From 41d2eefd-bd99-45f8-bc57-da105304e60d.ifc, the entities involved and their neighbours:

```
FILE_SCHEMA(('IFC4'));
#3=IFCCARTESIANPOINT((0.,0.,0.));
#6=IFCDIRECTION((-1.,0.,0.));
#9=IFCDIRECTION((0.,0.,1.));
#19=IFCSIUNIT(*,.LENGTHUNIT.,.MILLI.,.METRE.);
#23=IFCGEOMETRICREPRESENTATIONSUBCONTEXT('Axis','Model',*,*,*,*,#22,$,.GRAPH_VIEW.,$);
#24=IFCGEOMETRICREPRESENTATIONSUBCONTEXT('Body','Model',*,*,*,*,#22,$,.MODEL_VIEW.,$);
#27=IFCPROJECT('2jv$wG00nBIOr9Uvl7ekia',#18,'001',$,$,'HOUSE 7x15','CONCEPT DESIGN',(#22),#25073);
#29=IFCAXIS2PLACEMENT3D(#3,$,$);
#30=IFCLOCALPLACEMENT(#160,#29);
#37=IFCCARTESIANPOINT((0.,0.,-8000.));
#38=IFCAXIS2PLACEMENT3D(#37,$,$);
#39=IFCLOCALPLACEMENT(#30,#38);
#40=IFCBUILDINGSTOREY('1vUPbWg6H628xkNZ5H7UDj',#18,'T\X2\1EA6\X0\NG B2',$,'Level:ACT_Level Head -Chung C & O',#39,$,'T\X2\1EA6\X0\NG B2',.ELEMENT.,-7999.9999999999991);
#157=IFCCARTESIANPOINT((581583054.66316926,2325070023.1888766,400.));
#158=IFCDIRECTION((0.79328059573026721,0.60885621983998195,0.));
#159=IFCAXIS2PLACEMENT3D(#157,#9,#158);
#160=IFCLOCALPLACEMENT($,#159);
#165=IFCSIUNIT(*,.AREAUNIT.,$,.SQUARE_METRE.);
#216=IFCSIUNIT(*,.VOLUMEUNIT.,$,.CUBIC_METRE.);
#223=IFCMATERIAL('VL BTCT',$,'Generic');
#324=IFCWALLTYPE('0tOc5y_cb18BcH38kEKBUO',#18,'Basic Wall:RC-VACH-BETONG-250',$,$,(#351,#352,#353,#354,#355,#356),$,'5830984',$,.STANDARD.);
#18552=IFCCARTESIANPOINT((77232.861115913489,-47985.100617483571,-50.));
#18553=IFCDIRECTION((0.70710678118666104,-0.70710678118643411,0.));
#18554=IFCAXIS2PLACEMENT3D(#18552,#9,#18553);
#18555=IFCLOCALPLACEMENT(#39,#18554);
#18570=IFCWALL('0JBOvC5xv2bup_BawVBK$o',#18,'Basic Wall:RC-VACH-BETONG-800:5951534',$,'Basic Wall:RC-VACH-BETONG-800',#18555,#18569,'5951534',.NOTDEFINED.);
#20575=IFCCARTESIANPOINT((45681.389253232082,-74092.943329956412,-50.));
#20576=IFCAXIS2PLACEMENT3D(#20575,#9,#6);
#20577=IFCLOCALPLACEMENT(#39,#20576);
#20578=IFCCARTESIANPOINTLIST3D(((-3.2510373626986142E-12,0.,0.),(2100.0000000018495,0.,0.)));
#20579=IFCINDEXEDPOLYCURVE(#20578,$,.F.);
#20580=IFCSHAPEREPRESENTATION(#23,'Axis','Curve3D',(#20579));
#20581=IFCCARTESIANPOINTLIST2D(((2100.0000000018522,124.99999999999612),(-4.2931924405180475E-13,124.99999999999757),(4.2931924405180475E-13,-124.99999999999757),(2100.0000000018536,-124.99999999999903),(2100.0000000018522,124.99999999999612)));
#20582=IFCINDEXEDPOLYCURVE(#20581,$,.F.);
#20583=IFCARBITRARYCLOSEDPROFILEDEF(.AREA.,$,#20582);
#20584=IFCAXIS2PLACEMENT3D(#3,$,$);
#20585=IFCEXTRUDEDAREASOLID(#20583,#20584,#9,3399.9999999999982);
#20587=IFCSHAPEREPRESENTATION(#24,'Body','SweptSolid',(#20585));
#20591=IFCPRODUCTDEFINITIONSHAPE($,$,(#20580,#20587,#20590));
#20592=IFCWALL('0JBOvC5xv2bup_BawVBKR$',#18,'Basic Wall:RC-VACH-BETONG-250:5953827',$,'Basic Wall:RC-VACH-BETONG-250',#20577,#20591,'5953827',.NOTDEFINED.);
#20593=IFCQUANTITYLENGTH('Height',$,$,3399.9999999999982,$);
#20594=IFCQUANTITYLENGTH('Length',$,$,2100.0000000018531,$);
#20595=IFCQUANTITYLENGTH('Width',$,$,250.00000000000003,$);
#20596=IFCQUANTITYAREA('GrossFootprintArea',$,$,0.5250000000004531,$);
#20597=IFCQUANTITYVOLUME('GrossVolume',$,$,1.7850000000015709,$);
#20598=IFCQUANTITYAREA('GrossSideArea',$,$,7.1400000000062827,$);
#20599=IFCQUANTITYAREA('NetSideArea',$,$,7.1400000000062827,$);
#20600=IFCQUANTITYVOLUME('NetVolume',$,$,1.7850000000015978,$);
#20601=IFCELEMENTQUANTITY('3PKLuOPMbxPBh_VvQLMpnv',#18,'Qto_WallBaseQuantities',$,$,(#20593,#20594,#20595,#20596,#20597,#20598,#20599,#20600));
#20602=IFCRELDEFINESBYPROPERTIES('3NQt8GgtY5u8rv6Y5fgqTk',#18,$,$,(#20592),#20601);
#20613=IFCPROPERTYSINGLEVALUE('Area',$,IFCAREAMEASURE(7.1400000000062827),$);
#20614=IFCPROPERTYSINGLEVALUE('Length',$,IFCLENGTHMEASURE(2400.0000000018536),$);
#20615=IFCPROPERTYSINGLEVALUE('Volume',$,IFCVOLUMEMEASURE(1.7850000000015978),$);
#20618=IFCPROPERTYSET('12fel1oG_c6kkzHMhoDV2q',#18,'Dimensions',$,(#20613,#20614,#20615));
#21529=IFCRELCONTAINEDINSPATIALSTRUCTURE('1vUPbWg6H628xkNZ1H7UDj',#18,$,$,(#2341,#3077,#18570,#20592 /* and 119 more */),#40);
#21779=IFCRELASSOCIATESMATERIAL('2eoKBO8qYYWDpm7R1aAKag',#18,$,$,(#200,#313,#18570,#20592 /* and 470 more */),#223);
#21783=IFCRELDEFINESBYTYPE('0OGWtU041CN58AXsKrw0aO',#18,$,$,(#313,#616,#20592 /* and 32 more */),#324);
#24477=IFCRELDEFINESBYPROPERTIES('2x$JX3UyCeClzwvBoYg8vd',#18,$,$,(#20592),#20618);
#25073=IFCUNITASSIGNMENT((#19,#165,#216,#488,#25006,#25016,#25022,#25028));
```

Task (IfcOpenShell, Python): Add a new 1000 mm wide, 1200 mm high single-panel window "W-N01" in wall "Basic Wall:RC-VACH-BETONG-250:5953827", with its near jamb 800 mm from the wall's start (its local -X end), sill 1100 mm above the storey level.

```python
import numpy as np
import ifcopenshell
import ifcopenshell.api.feature
import ifcopenshell.api.geometry
import ifcopenshell.api.pset
import ifcopenshell.api.root
import ifcopenshell.api.spatial
import ifcopenshell.geom
import ifcopenshell.util.element
import ifcopenshell.util.placement
import ifcopenshell.util.representation
import ifcopenshell.util.shape
import ifcopenshell.util.unit

model = ifcopenshell.open("41d2eefd-bd99-45f8-bc57-da105304e60d.ifc")
unit_scale = ifcopenshell.util.unit.calculate_unit_scale(model)
area_scale = ifcopenshell.util.unit.calculate_unit_scale(model, "AREAUNIT")
volume_scale = ifcopenshell.util.unit.calculate_unit_scale(model, "VOLUMEUNIT")
settings = ifcopenshell.geom.settings()


def volume(element):
    """Net volume in cubic metres, openings subtracted."""
    shape = ifcopenshell.geom.create_shape(settings, element)
    return ifcopenshell.util.shape.get_volume(shape.geometry)


wall = model.by_guid("0JBOvC5xv2bup_BawVBKR$")
storey = ifcopenshell.util.element.get_container(wall, ifc_class="IfcBuildingStorey")
context = ifcopenshell.util.representation.get_context(model, "Model", "Body", "MODEL_VIEW")
before = volume(wall)

width, height, from_end, sill = 1, 1.2, 0.8, 1.1  # metres

# The wall runs along its own X axis, and the end named is its -X end.
wall_shape = ifcopenshell.geom.create_shape(settings, wall)
x, y, z = ifcopenshell.util.shape.get_vertices(wall_shape.geometry).T
start = x.min() + from_end
face, thickness = float(y.min()), float(y.max() - y.min())
wall_matrix = ifcopenshell.util.placement.get_local_placement(wall.ObjectPlacement)
level = ifcopenshell.util.placement.get_local_placement(storey.ObjectPlacement)[2, 3]


def in_wall(x, y):
    """Placement at x, y metres in the wall's axes, at sill height."""
    matrix = wall_matrix.copy()
    matrix[:, 3] = wall_matrix @ np.array([x / unit_scale, y / unit_scale, 0.0, 1.0])
    matrix[2, 3] = level + sill / unit_scale
    return matrix


# Opening: a box that overshoots both wall faces by 50 mm.
opening = ifcopenshell.api.root.create_entity(model, ifc_class="IfcOpeningElement", predefined_type="OPENING")
box = ifcopenshell.api.geometry.add_wall_representation(
    model, context=context, length=width, height=height, thickness=thickness + 0.1
)
ifcopenshell.api.geometry.assign_representation(model, product=opening, representation=box)
ifcopenshell.api.geometry.edit_object_placement(model, product=opening, matrix=in_wall(start, face - 0.05), is_si=False)
ifcopenshell.api.feature.add_feature(model, feature=opening, element=wall)

window = ifcopenshell.api.root.create_entity(model, ifc_class="IfcWindow", name="W-N01", predefined_type="WINDOW")
window.OverallWidth, window.OverallHeight = width / unit_scale, height / unit_scale
window.PartitioningType = "SINGLE_PANEL"
body = ifcopenshell.api.geometry.add_window_representation(
    model,
    context=context,
    overall_width=window.OverallWidth,
    overall_height=window.OverallHeight,
    partition_type="SINGLE_PANEL",
)
ifcopenshell.api.geometry.assign_representation(model, product=window, representation=body)
ifcopenshell.api.spatial.assign_container(model, products=[window], relating_structure=storey)
ifcopenshell.api.feature.add_filling(model, opening=opening, element=window)

# Centre the window in the wall's thickness.
ifcopenshell.api.geometry.edit_object_placement(model, product=window, matrix=in_wall(start, face), is_si=False)
window_shape = ifcopenshell.geom.create_shape(settings, window)
depth = ifcopenshell.util.shape.get_vertices(window_shape.geometry)[:, 1]
offset = face + thickness / 2 - (depth.min() + depth.max()) / 2
ifcopenshell.api.geometry.edit_object_placement(model, product=window, matrix=in_wall(start, offset), is_si=False)

after = volume(wall)

# Update the wall's stored quantities.
qto = model.by_id(ifcopenshell.util.element.get_pset(wall, "Qto_WallBaseQuantities", should_inherit=False)["id"])
ifcopenshell.api.pset.edit_qto(model, qto=qto, properties={
    "NetSideArea": after / thickness / area_scale,
    "NetVolume": after / volume_scale,
})
pset = model.by_id(ifcopenshell.util.element.get_pset(wall, "Dimensions", should_inherit=False)["id"])
ifcopenshell.api.pset.edit_pset(model, pset=pset, properties={
    "Area": model.create_entity("IfcAreaMeasure", after / thickness / area_scale),
    "Volume": model.create_entity("IfcVolumeMeasure", after / volume_scale),
})

print(f"wall volume {before:.3f} -> {after:.3f} m3")

model.write("41d2eefd-bd99-45f8-bc57-da105304e60d-out.ifc")
```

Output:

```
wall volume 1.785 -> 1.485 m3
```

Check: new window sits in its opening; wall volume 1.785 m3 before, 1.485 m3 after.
